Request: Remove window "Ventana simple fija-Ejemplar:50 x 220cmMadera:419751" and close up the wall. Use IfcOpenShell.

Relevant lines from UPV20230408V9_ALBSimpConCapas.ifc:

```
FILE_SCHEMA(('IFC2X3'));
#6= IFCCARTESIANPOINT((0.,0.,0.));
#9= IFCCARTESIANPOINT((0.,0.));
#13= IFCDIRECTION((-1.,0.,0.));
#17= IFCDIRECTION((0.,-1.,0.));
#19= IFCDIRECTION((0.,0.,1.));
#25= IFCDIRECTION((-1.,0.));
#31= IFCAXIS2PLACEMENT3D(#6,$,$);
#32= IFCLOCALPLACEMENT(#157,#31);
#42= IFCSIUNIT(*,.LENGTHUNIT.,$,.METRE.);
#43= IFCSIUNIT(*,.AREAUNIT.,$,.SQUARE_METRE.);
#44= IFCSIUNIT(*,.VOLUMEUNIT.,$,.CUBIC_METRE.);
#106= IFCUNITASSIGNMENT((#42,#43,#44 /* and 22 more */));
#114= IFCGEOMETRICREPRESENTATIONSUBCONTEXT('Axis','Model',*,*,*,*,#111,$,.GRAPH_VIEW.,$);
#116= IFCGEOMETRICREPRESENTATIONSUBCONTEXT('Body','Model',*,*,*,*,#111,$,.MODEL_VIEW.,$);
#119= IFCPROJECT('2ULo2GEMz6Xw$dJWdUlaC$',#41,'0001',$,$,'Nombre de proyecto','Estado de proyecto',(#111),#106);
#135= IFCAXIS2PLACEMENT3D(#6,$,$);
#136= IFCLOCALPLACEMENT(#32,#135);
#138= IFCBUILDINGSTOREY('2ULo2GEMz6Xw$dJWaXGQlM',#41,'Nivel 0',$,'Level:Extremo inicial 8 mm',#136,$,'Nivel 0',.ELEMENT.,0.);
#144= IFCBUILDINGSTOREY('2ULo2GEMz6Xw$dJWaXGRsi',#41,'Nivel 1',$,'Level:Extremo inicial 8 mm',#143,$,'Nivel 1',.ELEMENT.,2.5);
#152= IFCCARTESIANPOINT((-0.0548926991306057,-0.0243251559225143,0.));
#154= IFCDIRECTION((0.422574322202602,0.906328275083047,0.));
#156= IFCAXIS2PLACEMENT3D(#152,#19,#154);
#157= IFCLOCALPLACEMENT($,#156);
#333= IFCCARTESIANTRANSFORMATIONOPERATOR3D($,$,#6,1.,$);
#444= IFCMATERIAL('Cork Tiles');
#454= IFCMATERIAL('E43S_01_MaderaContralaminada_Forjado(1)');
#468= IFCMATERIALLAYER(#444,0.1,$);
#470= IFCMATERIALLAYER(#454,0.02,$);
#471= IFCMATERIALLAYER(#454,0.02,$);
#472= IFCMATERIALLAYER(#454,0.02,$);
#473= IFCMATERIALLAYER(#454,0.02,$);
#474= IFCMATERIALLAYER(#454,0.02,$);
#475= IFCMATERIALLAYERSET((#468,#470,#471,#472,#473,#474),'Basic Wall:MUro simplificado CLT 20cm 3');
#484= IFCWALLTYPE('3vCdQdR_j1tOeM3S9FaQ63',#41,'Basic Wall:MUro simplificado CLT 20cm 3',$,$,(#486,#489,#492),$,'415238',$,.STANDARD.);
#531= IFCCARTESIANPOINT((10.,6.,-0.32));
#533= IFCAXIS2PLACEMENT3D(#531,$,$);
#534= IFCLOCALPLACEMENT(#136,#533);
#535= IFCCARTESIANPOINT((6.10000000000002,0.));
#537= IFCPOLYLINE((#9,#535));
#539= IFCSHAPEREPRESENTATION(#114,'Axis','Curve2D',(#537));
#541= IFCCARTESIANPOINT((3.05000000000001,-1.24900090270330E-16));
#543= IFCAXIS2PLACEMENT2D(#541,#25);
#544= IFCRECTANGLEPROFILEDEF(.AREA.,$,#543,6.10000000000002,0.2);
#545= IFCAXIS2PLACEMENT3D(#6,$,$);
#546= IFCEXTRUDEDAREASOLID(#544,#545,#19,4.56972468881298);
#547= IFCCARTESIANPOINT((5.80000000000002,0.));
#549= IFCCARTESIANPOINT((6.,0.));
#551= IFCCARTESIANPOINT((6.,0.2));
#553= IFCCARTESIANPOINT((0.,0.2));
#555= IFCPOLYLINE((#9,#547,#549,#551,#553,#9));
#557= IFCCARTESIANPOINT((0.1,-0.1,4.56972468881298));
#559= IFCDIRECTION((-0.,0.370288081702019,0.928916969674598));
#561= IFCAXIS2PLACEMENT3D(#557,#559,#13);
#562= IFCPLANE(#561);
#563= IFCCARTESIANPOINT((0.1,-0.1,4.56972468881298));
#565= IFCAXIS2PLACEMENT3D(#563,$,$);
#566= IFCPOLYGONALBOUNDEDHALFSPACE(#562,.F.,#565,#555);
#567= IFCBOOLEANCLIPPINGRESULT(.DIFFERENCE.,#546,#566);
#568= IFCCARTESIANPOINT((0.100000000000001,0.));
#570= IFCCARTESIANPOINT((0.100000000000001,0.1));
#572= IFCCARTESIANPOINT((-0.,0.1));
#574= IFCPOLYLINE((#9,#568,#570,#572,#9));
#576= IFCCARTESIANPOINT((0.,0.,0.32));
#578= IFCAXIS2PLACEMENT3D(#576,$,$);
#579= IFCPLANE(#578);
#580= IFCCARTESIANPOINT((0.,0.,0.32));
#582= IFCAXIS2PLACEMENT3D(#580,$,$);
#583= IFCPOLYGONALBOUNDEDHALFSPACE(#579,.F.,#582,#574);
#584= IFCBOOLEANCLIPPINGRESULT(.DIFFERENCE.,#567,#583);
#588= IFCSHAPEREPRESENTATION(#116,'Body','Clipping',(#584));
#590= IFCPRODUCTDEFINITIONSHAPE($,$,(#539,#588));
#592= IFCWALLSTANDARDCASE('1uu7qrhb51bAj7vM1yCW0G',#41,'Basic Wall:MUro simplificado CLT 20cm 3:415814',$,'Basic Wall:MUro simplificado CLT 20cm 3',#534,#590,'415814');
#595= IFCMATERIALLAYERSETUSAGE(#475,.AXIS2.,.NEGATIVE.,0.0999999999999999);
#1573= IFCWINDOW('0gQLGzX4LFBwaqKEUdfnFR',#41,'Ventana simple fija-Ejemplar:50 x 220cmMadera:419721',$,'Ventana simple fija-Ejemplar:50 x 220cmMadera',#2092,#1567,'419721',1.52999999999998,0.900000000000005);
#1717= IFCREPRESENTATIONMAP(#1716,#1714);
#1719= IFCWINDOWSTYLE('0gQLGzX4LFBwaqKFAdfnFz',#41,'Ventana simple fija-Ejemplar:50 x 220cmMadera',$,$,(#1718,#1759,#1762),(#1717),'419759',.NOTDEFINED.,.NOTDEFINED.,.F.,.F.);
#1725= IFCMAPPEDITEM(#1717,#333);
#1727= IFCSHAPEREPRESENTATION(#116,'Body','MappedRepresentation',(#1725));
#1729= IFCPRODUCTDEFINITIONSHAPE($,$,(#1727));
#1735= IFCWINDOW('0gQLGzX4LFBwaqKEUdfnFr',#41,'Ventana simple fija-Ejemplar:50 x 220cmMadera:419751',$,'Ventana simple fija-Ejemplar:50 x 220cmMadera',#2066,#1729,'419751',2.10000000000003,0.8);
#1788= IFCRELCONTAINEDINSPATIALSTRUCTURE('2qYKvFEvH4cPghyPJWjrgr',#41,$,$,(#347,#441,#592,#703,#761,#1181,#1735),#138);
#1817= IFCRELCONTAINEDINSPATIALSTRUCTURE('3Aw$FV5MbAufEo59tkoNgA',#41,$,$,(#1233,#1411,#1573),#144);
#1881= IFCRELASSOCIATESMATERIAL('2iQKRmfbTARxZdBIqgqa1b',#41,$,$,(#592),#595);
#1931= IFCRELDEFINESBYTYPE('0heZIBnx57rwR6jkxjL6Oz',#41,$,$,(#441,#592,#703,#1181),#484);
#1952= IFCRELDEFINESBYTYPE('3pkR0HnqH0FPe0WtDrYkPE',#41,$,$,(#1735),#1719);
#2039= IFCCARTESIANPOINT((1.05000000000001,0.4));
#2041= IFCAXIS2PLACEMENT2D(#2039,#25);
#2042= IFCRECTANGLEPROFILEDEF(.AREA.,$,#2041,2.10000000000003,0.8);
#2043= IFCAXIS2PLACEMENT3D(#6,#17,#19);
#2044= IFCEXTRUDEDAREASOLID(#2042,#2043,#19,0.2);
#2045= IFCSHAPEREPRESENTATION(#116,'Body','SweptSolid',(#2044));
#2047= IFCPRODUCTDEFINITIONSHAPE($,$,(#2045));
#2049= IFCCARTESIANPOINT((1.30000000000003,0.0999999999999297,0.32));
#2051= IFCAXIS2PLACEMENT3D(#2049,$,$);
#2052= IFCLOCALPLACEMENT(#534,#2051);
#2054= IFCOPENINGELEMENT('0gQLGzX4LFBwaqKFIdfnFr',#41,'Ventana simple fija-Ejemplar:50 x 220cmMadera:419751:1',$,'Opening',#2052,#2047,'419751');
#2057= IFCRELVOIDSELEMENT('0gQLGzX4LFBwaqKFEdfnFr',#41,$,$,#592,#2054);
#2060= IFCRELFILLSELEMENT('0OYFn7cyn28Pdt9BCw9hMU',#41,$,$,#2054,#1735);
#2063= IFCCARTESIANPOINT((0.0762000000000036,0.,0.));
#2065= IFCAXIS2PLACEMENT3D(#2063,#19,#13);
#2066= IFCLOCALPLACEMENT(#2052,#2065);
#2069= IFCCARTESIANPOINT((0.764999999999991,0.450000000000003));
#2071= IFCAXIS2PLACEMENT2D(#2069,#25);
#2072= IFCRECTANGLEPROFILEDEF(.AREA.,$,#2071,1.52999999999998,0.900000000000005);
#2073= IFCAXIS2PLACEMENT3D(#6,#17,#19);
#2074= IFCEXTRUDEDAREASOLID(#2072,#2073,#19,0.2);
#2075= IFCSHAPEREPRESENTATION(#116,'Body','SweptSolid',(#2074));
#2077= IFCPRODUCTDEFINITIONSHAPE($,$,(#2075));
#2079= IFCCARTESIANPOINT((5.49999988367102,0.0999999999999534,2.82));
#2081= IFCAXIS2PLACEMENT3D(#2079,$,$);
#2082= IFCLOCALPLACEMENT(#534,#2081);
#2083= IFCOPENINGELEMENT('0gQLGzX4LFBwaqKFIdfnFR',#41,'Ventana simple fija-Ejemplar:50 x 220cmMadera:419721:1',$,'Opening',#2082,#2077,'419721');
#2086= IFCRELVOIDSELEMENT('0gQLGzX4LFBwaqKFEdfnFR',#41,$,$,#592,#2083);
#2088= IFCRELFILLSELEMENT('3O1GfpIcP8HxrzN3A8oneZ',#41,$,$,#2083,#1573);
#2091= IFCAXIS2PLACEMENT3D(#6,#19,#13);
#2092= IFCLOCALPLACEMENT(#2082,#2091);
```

```python
import ifcopenshell
import ifcopenshell.api.feature
import ifcopenshell.api.root
import ifcopenshell.geom
import ifcopenshell.util.shape

model = ifcopenshell.open("UPV20230408V9_ALBSimpConCapas.ifc")
settings = ifcopenshell.geom.settings()


def volume(element):
    """Net volume in cubic metres, openings subtracted."""
    shape = ifcopenshell.geom.create_shape(settings, element)
    return ifcopenshell.util.shape.get_volume(shape.geometry)


window = model.by_guid("0gQLGzX4LFBwaqKEUdfnFr")
opening = window.FillsVoids[0].RelatingOpeningElement
wall = opening.VoidsElements[0].RelatingBuildingElement
before = volume(wall)

ifcopenshell.api.root.remove_product(model, product=window)
ifcopenshell.api.feature.remove_feature(model, feature=opening)

after = volume(wall)

print(f"wall volume {before:.3f} -> {after:.3f} m3")

model.write("UPV20230408V9_ALBSimpConCapas_updated.ifc")
```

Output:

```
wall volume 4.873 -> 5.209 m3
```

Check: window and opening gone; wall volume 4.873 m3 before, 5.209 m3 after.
